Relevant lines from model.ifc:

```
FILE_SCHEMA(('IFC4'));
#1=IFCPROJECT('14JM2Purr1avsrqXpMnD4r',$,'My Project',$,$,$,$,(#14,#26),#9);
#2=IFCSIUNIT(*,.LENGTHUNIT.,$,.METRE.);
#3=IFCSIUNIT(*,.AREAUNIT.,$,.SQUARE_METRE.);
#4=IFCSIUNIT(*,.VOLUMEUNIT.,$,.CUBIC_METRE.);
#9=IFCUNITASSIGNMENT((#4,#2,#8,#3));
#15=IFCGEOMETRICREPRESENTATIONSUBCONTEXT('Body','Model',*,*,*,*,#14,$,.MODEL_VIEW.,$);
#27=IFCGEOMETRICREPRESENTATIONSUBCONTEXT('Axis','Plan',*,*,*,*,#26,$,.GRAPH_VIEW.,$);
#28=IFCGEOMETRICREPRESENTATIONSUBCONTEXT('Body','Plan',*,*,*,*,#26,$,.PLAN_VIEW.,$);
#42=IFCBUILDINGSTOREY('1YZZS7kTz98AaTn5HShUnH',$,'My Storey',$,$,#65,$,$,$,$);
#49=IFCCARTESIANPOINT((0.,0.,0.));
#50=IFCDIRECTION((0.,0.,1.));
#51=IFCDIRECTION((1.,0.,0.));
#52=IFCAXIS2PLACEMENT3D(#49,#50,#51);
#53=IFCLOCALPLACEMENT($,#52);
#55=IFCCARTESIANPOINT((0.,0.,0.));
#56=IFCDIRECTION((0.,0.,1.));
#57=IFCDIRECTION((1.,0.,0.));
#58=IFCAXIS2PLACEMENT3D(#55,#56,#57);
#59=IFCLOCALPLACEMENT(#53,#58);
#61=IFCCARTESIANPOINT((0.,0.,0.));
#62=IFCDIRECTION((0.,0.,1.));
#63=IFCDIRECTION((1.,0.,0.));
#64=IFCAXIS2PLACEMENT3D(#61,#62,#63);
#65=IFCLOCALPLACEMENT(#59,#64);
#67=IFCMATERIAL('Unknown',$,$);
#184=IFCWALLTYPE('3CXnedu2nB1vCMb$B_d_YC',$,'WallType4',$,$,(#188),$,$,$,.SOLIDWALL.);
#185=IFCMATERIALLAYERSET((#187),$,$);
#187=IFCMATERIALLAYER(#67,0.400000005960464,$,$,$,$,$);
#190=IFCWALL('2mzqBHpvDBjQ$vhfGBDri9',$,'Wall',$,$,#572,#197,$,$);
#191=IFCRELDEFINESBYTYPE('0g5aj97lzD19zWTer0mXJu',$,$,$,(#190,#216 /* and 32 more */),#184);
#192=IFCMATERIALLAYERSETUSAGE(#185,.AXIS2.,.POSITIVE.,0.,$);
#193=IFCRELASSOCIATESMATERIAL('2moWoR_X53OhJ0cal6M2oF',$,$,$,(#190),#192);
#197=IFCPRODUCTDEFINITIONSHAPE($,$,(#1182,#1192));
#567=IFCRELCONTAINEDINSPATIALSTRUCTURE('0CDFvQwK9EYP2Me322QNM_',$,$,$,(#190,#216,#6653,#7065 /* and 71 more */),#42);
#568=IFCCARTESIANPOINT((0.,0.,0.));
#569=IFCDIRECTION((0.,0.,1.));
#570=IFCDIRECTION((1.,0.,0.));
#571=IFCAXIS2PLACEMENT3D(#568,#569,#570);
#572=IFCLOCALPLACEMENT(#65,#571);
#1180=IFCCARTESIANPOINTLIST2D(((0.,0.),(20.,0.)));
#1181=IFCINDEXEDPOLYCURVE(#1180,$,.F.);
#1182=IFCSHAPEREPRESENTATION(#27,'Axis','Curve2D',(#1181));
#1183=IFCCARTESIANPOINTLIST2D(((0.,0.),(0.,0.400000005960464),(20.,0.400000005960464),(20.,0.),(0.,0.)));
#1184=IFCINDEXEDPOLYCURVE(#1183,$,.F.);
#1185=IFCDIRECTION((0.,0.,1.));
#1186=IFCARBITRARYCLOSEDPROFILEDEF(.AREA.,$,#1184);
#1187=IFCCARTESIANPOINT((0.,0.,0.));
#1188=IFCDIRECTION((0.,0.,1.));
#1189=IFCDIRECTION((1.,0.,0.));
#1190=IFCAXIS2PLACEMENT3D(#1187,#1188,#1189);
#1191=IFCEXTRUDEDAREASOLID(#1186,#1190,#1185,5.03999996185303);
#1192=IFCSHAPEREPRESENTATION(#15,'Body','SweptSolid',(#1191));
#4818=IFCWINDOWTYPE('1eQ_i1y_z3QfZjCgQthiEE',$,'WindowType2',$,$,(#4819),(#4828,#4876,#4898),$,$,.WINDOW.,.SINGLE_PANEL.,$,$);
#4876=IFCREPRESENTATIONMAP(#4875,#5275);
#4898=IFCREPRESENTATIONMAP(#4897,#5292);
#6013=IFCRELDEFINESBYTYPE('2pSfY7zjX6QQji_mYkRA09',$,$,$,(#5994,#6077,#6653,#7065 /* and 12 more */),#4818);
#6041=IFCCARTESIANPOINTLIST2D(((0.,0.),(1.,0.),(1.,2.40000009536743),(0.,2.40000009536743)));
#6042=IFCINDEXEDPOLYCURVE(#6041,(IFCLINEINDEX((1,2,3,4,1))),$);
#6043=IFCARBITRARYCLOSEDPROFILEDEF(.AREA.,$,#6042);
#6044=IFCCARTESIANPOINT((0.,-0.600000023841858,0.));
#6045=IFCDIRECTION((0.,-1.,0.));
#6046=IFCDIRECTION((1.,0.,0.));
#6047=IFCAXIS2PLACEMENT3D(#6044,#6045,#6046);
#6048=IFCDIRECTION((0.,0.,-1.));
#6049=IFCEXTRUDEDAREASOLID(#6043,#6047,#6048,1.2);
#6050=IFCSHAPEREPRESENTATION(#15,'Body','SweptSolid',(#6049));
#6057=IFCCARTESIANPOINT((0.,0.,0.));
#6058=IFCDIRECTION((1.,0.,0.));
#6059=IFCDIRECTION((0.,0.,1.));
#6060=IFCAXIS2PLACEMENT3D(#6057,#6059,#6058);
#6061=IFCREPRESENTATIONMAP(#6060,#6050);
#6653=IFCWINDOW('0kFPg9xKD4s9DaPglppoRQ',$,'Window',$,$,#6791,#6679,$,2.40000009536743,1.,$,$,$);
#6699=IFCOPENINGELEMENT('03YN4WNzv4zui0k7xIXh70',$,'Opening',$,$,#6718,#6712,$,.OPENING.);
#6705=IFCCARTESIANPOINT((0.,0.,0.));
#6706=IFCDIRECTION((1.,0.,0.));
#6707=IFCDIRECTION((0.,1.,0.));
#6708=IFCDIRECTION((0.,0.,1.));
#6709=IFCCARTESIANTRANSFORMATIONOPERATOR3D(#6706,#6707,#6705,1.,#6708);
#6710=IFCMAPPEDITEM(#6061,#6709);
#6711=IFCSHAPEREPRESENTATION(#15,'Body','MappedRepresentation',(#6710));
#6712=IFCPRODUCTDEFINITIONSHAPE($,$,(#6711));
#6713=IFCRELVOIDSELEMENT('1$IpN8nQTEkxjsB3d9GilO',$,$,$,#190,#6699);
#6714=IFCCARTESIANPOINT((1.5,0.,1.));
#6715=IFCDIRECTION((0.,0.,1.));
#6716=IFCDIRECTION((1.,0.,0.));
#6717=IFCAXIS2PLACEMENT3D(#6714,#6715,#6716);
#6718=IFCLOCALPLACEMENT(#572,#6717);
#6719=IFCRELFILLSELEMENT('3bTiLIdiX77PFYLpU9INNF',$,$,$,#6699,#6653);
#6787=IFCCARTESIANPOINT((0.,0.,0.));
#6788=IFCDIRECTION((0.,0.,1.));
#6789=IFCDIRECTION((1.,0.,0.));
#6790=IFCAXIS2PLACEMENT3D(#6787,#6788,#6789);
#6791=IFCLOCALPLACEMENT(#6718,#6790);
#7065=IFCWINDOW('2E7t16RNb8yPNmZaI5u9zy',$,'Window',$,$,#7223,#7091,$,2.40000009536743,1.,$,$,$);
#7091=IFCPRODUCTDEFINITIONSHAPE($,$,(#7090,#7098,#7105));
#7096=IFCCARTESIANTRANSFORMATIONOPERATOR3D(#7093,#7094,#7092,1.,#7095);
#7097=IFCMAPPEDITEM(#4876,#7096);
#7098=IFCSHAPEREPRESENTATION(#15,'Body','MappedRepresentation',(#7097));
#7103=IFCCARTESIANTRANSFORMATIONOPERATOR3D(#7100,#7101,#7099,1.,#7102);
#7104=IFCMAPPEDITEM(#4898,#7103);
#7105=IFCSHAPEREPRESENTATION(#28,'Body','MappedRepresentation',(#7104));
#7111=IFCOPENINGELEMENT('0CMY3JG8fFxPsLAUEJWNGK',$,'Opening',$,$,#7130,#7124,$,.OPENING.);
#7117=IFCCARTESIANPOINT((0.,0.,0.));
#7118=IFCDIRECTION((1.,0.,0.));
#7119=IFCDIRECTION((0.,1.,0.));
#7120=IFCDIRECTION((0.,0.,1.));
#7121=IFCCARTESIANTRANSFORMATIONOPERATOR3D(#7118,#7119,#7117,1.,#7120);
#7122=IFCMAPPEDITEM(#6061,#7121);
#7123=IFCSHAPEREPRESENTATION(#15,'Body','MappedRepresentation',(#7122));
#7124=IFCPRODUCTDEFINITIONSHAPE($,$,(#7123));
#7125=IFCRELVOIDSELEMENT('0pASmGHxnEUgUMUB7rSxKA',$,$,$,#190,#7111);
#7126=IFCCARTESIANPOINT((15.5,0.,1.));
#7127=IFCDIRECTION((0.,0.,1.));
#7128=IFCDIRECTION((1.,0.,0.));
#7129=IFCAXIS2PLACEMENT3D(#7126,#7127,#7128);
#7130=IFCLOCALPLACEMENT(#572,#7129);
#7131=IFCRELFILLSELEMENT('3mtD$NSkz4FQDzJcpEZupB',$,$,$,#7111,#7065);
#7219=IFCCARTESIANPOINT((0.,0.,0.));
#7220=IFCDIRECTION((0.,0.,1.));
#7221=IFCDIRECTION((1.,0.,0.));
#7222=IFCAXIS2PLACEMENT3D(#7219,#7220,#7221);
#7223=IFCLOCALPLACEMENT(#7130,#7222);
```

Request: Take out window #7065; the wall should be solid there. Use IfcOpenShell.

```python
import ifcopenshell
import ifcopenshell.api.feature
import ifcopenshell.api.root
import ifcopenshell.geom
import ifcopenshell.util.shape

model = ifcopenshell.open("model.ifc")
settings = ifcopenshell.geom.settings()


def volume(element):
    """Net volume in cubic metres, openings subtracted."""
    shape = ifcopenshell.geom.create_shape(settings, element)
    return ifcopenshell.util.shape.get_volume(shape.geometry)


window = model.by_id(7065)
opening = window.FillsVoids[0].RelatingOpeningElement
wall = opening.VoidsElements[0].RelatingBuildingElement
before = volume(wall)

ifcopenshell.api.root.remove_product(model, product=window)
ifcopenshell.api.feature.remove_feature(model, feature=opening)

after = volume(wall)

print(f"wall volume {before:.3f} -> {after:.3f} m3")

model.write("model_updated.ifc")
```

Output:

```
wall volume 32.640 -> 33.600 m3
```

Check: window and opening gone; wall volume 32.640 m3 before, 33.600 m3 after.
